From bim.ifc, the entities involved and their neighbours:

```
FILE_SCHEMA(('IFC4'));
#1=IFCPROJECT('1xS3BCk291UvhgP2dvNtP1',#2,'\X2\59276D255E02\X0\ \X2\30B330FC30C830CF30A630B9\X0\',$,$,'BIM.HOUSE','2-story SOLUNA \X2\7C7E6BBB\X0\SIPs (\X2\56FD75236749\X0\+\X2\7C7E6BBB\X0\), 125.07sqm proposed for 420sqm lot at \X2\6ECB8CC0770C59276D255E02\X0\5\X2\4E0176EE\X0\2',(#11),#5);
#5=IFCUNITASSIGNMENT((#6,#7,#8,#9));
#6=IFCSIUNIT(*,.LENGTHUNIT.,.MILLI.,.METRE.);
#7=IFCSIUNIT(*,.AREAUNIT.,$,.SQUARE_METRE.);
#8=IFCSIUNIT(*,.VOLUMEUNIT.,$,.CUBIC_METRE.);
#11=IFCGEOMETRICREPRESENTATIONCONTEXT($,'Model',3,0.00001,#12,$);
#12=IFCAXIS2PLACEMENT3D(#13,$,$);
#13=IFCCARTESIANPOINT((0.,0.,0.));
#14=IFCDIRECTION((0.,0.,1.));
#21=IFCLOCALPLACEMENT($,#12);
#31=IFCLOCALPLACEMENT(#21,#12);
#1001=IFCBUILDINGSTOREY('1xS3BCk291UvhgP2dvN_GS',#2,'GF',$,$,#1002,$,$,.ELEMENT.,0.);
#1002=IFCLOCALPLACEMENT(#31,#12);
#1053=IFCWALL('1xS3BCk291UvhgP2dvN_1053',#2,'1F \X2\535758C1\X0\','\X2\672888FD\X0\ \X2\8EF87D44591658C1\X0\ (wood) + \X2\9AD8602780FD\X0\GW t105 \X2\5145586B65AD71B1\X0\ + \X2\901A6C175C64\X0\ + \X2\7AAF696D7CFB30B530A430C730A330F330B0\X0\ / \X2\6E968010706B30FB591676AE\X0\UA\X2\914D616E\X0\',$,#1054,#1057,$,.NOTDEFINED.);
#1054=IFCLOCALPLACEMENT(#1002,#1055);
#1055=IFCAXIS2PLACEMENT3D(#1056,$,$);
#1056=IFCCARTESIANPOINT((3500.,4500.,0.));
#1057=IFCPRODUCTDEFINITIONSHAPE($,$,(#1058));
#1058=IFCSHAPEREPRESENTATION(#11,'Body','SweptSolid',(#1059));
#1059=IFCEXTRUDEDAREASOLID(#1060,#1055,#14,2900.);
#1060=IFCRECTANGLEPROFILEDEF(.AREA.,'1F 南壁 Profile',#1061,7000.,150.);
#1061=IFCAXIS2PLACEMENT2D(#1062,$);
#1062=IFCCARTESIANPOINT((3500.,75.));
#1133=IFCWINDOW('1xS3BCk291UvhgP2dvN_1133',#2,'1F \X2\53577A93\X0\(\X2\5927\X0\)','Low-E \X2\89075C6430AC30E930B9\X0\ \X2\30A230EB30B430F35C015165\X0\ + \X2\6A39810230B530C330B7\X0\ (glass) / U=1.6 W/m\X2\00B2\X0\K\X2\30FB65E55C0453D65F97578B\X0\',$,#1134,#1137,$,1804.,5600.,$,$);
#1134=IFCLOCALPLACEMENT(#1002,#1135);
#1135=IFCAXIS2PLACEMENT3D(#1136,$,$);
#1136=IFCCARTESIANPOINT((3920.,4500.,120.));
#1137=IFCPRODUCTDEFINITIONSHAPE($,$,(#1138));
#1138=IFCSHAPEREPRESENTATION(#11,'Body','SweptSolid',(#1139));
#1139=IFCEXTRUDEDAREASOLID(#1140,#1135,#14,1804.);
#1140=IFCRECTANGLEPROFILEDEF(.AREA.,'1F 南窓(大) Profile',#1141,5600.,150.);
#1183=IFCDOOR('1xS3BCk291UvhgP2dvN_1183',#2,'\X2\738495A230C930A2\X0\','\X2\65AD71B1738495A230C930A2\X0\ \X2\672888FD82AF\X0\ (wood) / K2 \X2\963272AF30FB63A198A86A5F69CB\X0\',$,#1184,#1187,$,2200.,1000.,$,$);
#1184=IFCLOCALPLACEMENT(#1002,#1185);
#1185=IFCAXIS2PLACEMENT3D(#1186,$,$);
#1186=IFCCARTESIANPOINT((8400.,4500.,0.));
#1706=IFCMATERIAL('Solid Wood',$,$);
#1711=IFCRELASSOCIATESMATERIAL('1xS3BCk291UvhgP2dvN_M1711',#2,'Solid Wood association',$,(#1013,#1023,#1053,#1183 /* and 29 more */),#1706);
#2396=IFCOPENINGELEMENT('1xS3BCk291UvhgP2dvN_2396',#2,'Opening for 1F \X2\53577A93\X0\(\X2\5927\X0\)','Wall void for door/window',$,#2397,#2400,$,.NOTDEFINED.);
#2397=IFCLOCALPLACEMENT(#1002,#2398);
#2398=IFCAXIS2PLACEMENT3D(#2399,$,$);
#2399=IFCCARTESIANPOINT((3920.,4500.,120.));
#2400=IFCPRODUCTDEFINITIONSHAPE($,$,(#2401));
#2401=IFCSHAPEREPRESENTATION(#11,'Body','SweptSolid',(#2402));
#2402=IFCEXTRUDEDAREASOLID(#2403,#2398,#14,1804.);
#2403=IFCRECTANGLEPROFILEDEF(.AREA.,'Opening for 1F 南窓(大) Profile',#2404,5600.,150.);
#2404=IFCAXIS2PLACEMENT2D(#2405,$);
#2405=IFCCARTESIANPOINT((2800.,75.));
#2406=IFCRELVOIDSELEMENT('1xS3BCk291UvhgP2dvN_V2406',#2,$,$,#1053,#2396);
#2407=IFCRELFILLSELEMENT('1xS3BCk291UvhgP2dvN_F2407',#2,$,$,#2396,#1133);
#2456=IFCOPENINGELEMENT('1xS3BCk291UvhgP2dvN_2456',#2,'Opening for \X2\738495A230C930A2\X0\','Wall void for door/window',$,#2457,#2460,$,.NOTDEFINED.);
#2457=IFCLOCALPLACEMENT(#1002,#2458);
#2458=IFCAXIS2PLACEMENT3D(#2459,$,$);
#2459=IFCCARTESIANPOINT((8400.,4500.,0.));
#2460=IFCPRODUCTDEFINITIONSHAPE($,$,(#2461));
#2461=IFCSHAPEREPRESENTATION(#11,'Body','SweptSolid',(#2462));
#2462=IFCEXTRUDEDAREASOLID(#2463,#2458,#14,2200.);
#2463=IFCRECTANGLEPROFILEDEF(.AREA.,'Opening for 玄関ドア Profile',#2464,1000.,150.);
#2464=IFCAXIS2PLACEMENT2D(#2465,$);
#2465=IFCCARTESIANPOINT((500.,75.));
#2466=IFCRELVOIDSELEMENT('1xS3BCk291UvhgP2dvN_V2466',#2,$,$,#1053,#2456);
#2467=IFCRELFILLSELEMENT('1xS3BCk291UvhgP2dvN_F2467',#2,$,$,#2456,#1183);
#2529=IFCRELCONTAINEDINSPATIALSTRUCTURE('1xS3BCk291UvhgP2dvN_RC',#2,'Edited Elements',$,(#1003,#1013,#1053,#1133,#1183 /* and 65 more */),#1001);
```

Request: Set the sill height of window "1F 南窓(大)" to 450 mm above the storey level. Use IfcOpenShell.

```python
import numpy as np
import ifcopenshell
import ifcopenshell.api.geometry
import ifcopenshell.geom
import ifcopenshell.util.element
import ifcopenshell.util.placement
import ifcopenshell.util.shape
import ifcopenshell.util.unit

model = ifcopenshell.open("bim.ifc")
unit_scale = ifcopenshell.util.unit.calculate_unit_scale(model)

window = model.by_guid("1xS3BCk291UvhgP2dvN_1133")
opening = window.FillsVoids[0].RelatingOpeningElement
storey = ifcopenshell.util.element.get_container(window, ifc_class="IfcBuildingStorey")
level = ifcopenshell.util.placement.get_local_placement(storey.ObjectPlacement)[2, 3]

# The opening's origin need not be at the sill, so measure its lowest point.
shape = ifcopenshell.geom.create_shape(ifcopenshell.geom.settings(), opening)
bottom = ifcopenshell.util.shape.get_shape_bottom_elevation(shape, shape.geometry) / unit_scale
dz = level + 0.45 / unit_scale - bottom

shift = np.array([0.0, 0.0, dz])
# The window is not placed relative to its opening, so move both.
for product in (opening, window):
    matrix = ifcopenshell.util.placement.get_local_placement(product.ObjectPlacement)
    matrix[:3, 3] += shift
    ifcopenshell.api.geometry.edit_object_placement(model, product=product, matrix=matrix, is_si=False)

print(f"moved by {dz * unit_scale:+.3f} m")

model.write("bim_rev.ifc")
```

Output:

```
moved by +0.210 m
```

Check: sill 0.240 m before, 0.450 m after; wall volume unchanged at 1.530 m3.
